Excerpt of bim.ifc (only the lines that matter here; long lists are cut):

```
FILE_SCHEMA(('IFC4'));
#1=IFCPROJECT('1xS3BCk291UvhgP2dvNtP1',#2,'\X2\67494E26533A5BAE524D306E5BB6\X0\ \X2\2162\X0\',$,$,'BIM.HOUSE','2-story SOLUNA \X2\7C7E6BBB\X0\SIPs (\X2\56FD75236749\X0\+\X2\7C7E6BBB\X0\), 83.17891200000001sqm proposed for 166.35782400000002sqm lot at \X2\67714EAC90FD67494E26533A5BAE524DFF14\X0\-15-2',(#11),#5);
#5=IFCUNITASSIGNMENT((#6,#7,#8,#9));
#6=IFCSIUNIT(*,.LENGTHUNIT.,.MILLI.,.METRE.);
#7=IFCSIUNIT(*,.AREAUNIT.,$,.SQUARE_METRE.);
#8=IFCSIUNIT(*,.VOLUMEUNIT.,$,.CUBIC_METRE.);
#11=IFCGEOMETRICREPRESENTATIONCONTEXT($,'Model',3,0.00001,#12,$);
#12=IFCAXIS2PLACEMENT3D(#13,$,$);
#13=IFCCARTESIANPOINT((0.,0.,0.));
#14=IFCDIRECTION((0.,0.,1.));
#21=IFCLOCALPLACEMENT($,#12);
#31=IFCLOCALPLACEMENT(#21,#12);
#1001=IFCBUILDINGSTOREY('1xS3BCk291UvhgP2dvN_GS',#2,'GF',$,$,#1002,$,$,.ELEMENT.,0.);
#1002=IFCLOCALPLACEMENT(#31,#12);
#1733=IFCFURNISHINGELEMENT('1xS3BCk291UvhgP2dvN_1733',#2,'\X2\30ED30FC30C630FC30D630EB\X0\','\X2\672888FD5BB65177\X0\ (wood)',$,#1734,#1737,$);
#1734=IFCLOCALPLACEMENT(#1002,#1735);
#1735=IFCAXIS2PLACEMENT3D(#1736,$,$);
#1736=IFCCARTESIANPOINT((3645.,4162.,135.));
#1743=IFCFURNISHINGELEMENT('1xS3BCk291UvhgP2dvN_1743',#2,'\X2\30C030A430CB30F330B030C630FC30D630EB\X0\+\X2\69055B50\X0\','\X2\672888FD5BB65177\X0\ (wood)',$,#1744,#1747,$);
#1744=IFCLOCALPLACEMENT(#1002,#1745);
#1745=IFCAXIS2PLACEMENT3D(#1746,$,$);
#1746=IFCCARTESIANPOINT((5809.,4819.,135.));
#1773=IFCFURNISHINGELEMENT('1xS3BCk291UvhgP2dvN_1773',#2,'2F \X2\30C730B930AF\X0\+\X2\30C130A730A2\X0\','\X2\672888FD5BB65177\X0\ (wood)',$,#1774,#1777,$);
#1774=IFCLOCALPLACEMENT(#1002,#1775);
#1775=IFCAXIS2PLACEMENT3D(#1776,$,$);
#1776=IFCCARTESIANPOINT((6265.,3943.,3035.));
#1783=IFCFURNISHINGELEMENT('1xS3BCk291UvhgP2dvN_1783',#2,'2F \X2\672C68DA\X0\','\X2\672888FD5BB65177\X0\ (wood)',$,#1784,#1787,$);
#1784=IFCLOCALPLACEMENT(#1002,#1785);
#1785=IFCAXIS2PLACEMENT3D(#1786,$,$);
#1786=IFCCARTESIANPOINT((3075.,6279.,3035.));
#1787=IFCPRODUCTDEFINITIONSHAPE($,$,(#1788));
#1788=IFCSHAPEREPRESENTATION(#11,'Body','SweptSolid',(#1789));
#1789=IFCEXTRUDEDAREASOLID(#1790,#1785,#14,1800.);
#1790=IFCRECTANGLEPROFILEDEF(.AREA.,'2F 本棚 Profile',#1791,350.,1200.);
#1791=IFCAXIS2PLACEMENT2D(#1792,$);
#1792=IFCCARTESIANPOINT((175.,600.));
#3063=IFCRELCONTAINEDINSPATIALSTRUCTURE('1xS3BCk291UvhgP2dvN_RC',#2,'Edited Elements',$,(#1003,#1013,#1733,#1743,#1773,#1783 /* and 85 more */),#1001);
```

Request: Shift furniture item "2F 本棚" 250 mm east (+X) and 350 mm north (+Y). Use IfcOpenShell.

```python
import ifcopenshell
import ifcopenshell.api.geometry
import ifcopenshell.util.placement
import ifcopenshell.util.unit

model = ifcopenshell.open("bim.ifc")
unit_scale = ifcopenshell.util.unit.calculate_unit_scale(model)

item = model.by_guid("1xS3BCk291UvhgP2dvN_1783")
matrix = ifcopenshell.util.placement.get_local_placement(item.ObjectPlacement)
matrix[0, 3] += 0.25 / unit_scale
matrix[1, 3] += 0.35 / unit_scale
ifcopenshell.api.geometry.edit_object_placement(model, product=item, matrix=matrix, is_si=False)

print(ifcopenshell.util.placement.get_local_placement(item.ObjectPlacement).round(3) + 0.0)

model.write("bim_updated.ifc")
```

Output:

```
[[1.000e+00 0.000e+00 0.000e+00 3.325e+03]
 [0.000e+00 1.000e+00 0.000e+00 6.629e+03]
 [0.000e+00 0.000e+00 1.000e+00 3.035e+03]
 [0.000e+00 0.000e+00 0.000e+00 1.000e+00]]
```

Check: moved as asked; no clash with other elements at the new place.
